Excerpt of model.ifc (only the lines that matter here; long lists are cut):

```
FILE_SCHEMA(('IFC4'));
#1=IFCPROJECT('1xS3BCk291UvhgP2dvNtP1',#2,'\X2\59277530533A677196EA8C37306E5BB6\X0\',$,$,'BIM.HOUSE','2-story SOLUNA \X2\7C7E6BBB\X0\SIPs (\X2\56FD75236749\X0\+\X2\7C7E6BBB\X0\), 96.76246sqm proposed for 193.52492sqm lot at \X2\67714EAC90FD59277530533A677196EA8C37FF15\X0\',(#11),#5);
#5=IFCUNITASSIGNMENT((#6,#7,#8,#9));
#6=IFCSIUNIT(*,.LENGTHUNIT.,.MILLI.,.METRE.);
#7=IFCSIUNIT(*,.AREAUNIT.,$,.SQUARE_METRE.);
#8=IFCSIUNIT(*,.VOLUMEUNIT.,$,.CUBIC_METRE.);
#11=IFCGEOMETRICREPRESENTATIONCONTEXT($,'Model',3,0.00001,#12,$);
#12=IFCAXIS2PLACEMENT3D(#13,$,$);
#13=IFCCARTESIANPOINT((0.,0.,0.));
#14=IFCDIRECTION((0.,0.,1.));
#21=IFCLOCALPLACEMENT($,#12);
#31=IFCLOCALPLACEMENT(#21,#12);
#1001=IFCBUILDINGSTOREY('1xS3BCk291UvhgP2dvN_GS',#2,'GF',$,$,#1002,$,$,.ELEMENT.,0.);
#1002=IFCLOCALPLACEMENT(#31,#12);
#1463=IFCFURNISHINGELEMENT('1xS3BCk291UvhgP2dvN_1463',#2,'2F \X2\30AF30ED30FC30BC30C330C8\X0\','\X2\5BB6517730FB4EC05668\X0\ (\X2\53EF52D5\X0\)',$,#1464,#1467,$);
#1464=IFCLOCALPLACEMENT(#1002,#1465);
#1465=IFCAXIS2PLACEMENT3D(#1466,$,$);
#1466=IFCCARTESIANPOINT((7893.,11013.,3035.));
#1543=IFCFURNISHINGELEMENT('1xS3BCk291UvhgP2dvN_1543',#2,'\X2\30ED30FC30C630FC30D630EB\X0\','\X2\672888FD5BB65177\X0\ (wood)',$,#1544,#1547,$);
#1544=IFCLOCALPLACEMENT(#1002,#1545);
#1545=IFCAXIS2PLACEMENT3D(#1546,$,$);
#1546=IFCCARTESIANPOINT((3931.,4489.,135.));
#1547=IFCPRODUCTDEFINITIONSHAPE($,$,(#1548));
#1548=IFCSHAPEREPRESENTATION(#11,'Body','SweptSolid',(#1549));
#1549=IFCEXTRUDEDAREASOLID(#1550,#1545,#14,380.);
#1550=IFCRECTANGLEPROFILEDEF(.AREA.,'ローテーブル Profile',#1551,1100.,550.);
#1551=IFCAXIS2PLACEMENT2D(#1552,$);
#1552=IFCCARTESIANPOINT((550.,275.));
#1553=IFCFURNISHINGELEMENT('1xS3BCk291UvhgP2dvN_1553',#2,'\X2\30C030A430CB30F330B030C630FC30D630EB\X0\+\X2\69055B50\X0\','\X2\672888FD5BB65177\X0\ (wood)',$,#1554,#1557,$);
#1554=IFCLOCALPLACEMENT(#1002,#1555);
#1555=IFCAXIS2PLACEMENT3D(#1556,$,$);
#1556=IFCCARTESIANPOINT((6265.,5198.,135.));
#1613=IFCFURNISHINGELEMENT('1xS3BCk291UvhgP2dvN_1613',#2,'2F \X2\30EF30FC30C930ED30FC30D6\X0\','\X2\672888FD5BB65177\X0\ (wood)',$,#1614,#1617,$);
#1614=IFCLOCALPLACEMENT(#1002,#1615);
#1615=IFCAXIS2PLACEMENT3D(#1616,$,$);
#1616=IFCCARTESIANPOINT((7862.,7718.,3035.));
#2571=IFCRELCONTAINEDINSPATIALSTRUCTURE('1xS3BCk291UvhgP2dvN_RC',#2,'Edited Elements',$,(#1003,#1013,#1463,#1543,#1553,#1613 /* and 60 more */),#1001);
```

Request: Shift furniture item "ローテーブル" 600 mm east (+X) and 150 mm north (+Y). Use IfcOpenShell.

```python
import ifcopenshell
import ifcopenshell.api.geometry
import ifcopenshell.util.placement

model = ifcopenshell.open("model.ifc")

item = model.by_guid("1xS3BCk291UvhgP2dvN_1543")
matrix = ifcopenshell.util.placement.get_local_placement(item.ObjectPlacement)
matrix[0, 3] += 600.0
matrix[1, 3] += 150.0
ifcopenshell.api.geometry.edit_object_placement(model, product=item, matrix=matrix, is_si=False)

print(ifcopenshell.util.placement.get_local_placement(item.ObjectPlacement).round(3) + 0.0)

model.write("model_edited.ifc")
```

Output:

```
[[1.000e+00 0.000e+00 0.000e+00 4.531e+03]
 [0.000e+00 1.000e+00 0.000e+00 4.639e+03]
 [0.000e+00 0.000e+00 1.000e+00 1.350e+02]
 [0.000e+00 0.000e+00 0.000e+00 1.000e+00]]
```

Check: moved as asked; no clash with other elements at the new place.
